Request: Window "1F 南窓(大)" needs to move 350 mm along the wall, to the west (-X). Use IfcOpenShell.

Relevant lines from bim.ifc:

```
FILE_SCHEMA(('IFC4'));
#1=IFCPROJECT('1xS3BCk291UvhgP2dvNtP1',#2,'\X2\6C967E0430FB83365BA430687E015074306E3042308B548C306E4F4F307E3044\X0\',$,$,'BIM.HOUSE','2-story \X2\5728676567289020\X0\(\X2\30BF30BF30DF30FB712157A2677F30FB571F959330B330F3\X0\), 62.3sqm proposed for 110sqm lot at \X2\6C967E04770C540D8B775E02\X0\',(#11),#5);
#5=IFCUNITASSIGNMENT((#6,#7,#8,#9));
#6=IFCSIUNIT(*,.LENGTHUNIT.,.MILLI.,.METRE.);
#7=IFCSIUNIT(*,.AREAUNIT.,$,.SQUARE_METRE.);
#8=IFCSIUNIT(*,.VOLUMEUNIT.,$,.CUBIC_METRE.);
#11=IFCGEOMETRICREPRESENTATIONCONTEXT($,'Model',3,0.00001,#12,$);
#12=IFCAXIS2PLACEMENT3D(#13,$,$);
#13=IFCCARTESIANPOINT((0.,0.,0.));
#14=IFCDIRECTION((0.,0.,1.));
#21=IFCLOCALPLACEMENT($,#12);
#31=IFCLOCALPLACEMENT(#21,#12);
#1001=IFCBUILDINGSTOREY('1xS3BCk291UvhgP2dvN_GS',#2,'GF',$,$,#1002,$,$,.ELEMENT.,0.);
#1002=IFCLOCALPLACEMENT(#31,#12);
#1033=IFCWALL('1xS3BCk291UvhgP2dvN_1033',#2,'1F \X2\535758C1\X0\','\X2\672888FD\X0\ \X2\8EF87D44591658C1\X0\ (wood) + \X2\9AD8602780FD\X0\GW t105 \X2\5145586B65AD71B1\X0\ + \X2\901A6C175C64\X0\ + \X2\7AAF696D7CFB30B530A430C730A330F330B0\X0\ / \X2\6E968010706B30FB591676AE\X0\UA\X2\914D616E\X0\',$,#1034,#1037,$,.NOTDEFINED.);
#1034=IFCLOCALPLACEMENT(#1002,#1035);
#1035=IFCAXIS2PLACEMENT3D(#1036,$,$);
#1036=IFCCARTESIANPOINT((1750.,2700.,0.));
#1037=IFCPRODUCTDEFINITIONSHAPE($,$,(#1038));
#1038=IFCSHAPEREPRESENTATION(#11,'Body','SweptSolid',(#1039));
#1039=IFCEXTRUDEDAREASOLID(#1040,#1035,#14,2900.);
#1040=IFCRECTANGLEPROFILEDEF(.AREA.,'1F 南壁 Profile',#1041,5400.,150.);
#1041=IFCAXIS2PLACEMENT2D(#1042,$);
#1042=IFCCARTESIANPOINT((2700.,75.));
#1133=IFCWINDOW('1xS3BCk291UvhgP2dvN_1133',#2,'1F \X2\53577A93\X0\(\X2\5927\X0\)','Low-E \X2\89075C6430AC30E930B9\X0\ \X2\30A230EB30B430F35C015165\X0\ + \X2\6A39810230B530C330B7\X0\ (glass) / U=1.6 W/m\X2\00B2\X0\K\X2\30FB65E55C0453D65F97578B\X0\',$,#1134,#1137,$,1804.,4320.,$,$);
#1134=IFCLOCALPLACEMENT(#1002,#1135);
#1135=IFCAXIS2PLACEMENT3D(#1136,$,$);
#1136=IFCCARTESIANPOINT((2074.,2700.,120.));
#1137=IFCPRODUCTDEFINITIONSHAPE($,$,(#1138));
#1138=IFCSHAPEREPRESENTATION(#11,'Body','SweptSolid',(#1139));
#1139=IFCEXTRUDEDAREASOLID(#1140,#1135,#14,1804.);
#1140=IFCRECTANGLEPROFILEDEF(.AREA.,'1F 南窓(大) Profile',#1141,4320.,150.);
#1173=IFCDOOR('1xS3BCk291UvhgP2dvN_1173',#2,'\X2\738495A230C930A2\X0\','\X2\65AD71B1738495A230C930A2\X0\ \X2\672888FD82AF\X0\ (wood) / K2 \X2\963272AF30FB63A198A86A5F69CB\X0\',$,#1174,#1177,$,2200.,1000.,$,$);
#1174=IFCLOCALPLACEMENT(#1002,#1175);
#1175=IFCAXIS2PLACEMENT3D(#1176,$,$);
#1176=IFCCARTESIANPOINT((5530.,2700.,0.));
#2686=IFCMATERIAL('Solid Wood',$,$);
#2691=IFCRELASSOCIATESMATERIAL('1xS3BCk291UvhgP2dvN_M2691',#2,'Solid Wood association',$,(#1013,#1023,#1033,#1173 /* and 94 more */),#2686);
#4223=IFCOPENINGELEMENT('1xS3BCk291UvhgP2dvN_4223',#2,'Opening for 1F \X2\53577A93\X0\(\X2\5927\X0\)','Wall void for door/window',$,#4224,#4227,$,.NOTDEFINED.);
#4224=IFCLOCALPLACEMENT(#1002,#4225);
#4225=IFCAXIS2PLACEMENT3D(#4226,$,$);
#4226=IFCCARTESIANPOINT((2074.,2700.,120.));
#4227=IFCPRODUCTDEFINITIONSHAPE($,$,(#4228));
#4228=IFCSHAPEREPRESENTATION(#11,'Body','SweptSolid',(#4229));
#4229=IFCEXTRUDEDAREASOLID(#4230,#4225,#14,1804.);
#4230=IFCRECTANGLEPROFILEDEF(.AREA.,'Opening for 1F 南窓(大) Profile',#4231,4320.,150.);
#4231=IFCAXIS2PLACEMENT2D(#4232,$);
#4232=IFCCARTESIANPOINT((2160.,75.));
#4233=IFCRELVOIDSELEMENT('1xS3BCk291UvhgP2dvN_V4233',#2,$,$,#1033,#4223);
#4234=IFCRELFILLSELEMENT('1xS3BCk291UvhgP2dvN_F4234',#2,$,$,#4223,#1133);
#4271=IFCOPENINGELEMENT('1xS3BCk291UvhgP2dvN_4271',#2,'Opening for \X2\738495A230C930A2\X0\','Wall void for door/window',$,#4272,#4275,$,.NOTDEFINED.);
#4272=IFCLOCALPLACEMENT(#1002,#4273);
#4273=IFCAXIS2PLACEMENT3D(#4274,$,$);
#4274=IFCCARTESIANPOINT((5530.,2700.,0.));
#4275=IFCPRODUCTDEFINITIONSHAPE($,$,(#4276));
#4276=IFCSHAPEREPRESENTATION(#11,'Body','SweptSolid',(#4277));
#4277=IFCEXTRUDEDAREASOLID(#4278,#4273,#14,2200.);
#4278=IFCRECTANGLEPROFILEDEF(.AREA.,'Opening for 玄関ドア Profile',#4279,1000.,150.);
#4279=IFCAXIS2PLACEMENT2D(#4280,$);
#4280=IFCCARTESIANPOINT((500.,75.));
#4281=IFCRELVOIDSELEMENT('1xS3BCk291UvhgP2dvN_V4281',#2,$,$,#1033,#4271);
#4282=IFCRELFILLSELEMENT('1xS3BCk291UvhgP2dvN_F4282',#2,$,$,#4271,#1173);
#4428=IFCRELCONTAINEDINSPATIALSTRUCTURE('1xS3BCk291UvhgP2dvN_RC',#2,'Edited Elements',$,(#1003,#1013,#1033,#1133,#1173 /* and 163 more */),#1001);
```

```python
import ifcopenshell
import ifcopenshell.api.geometry
import ifcopenshell.util.placement
import ifcopenshell.util.unit

model = ifcopenshell.open("bim.ifc")
unit_scale = ifcopenshell.util.unit.calculate_unit_scale(model)

window = model.by_guid("1xS3BCk291UvhgP2dvN_1133")
opening = window.FillsVoids[0].RelatingOpeningElement
wall = opening.VoidsElements[0].RelatingBuildingElement

wall_matrix = ifcopenshell.util.placement.get_local_placement(wall.ObjectPlacement)
shift = wall_matrix[:3, 0] * -0.35 / unit_scale
before = ifcopenshell.util.placement.get_local_placement(window.ObjectPlacement)[:3, 3].copy()

# The window is not placed relative to its opening, so move both.
for product in (opening, window):
    matrix = ifcopenshell.util.placement.get_local_placement(product.ObjectPlacement)
    matrix[:3, 3] += shift
    ifcopenshell.api.geometry.edit_object_placement(model, product=product, matrix=matrix, is_si=False)

after = ifcopenshell.util.placement.get_local_placement(window.ObjectPlacement)[:3, 3]
print("window moved by", (after - before).round(3) + 0.0)

model.write("bim_v2.ifc")
```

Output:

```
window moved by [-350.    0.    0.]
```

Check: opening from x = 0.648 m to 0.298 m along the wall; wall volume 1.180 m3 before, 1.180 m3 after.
